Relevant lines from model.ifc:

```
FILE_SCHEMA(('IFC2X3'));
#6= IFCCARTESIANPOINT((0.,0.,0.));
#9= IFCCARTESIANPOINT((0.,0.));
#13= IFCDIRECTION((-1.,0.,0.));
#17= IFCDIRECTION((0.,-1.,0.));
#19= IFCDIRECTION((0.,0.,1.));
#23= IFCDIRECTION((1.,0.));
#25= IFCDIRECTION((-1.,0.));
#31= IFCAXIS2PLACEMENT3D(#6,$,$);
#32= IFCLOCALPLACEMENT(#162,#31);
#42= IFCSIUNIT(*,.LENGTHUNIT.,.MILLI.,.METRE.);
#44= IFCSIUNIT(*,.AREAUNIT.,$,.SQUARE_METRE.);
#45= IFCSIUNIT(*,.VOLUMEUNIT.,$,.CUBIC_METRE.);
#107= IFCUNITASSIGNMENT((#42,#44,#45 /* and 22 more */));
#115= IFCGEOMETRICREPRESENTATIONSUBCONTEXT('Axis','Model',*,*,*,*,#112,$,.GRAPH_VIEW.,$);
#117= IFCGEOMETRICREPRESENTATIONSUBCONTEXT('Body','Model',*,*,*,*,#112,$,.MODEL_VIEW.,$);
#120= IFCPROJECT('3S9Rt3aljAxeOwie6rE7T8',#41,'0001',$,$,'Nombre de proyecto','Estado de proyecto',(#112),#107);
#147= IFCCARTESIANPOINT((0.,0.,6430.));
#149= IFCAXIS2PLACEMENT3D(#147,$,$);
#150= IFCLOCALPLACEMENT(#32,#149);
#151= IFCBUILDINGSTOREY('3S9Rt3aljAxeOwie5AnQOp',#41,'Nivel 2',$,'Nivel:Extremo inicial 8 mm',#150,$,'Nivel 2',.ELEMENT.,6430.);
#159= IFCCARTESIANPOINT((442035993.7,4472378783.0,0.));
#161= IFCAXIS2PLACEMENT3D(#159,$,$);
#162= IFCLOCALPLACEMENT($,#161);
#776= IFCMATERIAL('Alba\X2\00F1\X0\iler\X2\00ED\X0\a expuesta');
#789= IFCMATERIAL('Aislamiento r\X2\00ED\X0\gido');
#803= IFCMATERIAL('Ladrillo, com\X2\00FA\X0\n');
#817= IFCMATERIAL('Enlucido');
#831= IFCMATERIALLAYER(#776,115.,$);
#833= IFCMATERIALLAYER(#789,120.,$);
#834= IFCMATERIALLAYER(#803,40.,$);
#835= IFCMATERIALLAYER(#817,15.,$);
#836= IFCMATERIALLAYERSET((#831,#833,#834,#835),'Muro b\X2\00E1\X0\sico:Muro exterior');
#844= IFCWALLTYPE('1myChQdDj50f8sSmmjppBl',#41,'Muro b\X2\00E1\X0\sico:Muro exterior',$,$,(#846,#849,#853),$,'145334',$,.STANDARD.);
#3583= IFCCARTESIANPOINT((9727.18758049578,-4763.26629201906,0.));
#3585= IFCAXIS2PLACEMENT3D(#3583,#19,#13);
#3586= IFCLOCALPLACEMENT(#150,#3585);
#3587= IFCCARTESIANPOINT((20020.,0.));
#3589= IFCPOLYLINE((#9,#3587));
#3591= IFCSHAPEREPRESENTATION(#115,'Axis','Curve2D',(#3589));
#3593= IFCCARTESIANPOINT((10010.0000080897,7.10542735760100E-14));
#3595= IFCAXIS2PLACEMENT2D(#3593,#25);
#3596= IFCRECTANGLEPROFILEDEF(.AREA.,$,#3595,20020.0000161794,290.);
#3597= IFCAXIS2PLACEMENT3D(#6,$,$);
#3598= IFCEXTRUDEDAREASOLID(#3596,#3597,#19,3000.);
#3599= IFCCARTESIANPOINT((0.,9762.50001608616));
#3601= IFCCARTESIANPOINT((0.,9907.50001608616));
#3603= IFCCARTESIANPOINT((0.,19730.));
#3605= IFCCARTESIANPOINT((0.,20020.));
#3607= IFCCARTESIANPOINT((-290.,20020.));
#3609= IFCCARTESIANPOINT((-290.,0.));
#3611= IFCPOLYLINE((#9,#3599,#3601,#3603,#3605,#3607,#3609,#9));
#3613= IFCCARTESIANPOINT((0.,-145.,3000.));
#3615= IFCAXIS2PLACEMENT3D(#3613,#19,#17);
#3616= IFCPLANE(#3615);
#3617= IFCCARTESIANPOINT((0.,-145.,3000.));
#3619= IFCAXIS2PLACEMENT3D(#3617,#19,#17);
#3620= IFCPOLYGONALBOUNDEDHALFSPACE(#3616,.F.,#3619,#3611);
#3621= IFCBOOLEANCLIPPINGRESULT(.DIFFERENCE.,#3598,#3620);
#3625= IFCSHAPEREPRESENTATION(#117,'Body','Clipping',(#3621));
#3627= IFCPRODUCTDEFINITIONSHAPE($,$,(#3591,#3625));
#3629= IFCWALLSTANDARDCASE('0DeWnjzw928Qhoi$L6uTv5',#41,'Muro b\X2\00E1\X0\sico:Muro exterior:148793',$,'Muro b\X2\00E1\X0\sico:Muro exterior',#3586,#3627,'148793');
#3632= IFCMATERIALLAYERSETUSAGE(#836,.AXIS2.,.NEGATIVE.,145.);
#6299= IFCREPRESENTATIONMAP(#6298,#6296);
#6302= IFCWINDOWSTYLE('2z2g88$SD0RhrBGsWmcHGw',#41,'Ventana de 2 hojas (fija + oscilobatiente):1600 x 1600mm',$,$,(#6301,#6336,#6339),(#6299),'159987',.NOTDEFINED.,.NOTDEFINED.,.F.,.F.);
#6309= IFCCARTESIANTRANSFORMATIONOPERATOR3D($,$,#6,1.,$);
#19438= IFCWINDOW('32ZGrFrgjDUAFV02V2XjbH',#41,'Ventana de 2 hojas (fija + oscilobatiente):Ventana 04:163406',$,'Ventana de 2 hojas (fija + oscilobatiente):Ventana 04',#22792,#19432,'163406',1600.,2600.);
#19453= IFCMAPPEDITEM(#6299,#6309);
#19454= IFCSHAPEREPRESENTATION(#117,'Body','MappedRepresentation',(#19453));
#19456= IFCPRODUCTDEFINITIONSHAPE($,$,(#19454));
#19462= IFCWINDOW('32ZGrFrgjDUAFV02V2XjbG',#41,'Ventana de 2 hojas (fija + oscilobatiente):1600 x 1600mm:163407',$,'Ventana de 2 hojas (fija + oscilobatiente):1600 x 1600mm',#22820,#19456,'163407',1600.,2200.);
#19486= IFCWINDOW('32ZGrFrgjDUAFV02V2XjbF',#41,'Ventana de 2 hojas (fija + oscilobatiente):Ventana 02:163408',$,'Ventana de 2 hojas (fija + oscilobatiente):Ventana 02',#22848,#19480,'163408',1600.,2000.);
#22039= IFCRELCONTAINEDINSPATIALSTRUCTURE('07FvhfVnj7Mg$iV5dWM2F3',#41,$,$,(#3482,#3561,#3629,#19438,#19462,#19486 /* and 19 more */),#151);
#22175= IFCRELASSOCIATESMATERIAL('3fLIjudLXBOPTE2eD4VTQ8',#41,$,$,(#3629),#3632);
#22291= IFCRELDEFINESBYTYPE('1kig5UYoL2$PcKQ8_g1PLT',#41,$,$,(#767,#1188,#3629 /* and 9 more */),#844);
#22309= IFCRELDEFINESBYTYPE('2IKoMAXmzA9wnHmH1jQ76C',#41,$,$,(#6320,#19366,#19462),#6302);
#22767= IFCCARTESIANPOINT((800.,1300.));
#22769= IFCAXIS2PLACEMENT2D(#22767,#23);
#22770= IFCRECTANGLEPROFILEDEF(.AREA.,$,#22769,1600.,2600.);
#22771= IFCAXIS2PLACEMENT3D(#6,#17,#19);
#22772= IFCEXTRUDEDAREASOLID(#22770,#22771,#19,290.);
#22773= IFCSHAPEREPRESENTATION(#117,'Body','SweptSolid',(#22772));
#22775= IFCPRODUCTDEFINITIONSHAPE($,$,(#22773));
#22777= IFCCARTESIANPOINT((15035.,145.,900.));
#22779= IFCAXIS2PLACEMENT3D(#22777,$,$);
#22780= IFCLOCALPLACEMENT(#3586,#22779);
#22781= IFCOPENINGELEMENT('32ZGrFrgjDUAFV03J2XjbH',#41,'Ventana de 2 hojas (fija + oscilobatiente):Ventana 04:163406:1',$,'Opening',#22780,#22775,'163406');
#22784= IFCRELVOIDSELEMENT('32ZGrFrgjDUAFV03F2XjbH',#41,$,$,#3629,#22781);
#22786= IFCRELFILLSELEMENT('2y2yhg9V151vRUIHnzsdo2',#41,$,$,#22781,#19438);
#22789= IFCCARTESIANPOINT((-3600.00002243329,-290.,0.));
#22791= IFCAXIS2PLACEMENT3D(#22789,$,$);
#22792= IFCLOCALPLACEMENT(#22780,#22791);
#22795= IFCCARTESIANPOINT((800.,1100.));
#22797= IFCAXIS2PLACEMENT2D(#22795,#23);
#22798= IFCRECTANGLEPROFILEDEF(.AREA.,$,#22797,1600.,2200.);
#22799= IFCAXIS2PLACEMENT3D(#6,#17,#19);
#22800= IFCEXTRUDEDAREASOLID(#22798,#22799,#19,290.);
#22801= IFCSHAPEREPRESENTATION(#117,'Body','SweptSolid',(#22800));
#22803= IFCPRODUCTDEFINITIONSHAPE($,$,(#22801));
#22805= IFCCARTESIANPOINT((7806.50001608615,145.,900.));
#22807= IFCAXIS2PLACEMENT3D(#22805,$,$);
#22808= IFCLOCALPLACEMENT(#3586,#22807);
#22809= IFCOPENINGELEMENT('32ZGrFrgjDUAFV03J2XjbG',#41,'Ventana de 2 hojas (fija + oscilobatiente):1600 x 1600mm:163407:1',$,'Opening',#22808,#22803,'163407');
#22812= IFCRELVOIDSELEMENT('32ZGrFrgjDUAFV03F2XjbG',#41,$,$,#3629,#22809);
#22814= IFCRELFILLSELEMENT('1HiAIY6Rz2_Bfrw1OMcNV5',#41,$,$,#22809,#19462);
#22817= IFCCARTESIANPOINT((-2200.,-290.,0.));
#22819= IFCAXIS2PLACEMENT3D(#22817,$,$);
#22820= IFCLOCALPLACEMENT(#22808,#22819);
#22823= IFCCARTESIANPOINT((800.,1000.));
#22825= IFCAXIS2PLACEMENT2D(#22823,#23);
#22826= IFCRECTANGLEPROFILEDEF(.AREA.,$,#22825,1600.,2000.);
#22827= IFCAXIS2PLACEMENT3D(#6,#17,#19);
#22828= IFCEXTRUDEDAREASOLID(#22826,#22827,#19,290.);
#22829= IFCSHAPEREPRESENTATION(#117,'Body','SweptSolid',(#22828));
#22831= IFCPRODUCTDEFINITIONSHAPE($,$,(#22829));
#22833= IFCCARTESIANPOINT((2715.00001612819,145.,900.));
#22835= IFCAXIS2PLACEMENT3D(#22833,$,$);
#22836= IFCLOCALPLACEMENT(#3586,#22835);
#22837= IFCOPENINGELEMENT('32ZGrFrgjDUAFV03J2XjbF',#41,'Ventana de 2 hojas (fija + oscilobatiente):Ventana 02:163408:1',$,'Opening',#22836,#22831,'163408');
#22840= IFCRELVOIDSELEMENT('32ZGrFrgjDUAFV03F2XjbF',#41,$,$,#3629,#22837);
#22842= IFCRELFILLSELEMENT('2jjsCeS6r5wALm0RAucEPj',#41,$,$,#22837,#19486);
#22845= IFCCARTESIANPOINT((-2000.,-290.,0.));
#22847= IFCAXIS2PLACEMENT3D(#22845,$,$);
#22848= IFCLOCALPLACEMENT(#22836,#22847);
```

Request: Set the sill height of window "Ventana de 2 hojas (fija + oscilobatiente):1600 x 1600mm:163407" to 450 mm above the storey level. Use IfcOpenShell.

```python
import numpy as np
import ifcopenshell
import ifcopenshell.api.geometry
import ifcopenshell.geom
import ifcopenshell.util.element
import ifcopenshell.util.placement
import ifcopenshell.util.shape
import ifcopenshell.util.unit

model = ifcopenshell.open("model.ifc")
unit_scale = ifcopenshell.util.unit.calculate_unit_scale(model)

window = model.by_guid("32ZGrFrgjDUAFV02V2XjbG")
opening = window.FillsVoids[0].RelatingOpeningElement
storey = ifcopenshell.util.element.get_container(window, ifc_class="IfcBuildingStorey")
level = ifcopenshell.util.placement.get_local_placement(storey.ObjectPlacement)[2, 3]

# The opening's origin need not be at the sill, so measure its lowest point.
shape = ifcopenshell.geom.create_shape(ifcopenshell.geom.settings(), opening)
bottom = ifcopenshell.util.shape.get_shape_bottom_elevation(shape, shape.geometry) / unit_scale
dz = level + 0.45 / unit_scale - bottom

shift = np.array([0.0, 0.0, dz])
# The window is placed relative to its opening, so it follows when the opening moves.
matrix = ifcopenshell.util.placement.get_local_placement(opening.ObjectPlacement)
matrix[:3, 3] += shift
ifcopenshell.api.geometry.edit_object_placement(
    model, product=opening, matrix=matrix, is_si=False, should_transform_children=True
)

print(f"moved by {dz * unit_scale:+.3f} m")

model.write("model_updated.ifc")
```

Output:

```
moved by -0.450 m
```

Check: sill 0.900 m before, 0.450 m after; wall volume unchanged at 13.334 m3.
